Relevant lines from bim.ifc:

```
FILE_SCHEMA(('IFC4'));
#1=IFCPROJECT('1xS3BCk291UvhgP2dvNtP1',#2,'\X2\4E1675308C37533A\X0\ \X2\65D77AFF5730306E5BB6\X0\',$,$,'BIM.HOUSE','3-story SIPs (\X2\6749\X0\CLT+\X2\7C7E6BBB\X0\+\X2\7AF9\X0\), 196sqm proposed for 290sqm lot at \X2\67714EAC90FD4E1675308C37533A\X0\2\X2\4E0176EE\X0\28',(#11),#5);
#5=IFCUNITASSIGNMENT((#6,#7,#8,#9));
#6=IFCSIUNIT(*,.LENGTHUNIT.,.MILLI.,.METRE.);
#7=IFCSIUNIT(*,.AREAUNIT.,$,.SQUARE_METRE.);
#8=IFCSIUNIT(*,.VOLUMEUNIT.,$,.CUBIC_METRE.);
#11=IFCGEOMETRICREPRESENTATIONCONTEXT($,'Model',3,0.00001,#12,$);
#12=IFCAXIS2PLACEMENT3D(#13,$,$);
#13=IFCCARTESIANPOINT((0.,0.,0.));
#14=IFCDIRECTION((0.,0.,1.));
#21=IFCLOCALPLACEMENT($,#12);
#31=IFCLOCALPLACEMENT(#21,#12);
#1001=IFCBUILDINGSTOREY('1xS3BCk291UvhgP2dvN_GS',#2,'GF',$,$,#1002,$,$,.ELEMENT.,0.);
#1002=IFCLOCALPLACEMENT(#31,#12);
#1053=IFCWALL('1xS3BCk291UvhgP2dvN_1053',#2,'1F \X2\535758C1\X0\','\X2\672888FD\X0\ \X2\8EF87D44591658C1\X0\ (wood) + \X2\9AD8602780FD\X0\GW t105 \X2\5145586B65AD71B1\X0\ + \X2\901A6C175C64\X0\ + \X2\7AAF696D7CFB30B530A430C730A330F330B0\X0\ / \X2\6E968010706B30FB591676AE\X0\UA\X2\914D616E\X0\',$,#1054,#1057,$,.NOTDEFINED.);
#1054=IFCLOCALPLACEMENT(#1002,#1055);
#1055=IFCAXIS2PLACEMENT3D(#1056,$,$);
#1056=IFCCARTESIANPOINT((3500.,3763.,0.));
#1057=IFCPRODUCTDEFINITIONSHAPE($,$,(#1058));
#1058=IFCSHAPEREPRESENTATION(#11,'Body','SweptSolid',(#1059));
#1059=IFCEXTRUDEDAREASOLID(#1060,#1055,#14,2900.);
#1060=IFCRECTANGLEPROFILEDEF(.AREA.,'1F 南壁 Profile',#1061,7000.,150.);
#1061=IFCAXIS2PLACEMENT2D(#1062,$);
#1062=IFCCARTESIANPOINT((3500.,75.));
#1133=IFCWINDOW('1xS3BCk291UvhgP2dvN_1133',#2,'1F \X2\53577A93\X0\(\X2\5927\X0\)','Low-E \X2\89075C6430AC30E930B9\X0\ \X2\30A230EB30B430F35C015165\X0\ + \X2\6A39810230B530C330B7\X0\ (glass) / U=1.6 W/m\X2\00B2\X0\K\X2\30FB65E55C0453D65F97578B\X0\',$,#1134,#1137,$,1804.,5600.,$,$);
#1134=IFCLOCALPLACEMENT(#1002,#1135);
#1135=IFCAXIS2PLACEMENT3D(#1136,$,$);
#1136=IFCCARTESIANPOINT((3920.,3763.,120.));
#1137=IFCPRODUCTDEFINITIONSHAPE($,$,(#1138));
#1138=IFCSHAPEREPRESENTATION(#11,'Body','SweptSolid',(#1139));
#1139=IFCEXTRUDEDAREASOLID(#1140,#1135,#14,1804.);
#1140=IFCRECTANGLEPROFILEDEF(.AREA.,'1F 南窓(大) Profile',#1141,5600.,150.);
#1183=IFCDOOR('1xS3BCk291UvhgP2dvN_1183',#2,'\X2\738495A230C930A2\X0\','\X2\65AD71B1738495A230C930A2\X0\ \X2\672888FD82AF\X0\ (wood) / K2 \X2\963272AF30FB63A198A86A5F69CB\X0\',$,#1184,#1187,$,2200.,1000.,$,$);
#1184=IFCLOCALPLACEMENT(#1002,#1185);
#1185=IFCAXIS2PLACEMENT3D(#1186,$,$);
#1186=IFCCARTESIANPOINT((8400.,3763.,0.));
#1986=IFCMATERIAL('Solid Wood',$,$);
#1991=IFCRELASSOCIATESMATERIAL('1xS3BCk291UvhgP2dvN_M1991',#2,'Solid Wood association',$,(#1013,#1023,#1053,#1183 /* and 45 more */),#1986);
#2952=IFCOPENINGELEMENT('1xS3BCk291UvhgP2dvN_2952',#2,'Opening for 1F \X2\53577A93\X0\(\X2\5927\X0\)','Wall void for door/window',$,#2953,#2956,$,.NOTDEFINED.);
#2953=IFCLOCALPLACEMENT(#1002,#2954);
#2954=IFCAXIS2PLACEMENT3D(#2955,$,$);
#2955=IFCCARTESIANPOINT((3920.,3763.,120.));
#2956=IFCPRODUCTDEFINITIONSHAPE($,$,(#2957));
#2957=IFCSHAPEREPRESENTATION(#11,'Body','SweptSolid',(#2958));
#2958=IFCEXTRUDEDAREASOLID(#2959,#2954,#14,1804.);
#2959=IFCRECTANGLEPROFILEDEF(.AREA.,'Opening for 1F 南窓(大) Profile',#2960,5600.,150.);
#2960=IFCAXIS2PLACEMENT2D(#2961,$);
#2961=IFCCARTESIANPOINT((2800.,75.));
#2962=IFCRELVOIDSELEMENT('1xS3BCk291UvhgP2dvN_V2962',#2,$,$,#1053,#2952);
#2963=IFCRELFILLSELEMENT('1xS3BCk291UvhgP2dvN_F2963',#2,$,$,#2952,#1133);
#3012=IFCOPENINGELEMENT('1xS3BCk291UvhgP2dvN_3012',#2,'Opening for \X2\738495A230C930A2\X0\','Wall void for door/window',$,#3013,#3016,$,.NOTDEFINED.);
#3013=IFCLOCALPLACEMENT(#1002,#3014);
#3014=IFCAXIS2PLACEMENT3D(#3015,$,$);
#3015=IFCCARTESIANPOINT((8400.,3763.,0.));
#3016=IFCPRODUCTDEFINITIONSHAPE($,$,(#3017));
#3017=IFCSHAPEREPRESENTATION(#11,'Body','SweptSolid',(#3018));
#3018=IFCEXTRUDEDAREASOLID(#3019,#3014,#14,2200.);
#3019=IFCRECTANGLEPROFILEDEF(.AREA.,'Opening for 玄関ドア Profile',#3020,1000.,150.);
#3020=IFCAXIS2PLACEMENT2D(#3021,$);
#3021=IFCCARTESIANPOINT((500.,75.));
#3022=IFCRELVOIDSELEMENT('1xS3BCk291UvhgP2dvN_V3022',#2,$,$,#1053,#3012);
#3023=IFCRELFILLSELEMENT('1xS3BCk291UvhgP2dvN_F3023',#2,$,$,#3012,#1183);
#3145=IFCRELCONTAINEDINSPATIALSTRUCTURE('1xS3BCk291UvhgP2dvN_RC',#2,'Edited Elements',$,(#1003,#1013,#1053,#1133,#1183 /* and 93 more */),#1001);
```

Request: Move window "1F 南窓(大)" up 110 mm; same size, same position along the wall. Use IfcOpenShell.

```python
import numpy as np
import ifcopenshell
import ifcopenshell.api.geometry
import ifcopenshell.util.placement
import ifcopenshell.util.unit

model = ifcopenshell.open("bim.ifc")
unit_scale = ifcopenshell.util.unit.calculate_unit_scale(model)

window = model.by_guid("1xS3BCk291UvhgP2dvN_1133")
opening = window.FillsVoids[0].RelatingOpeningElement
dz = 110.0

shift = np.array([0.0, 0.0, dz])
# The window is not placed relative to its opening, so move both.
for product in (opening, window):
    matrix = ifcopenshell.util.placement.get_local_placement(product.ObjectPlacement)
    matrix[:3, 3] += shift
    ifcopenshell.api.geometry.edit_object_placement(model, product=product, matrix=matrix, is_si=False)

print(f"moved by {dz * unit_scale:+.3f} m")

model.write("bim-out.ifc")
```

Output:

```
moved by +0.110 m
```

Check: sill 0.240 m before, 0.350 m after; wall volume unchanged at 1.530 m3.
